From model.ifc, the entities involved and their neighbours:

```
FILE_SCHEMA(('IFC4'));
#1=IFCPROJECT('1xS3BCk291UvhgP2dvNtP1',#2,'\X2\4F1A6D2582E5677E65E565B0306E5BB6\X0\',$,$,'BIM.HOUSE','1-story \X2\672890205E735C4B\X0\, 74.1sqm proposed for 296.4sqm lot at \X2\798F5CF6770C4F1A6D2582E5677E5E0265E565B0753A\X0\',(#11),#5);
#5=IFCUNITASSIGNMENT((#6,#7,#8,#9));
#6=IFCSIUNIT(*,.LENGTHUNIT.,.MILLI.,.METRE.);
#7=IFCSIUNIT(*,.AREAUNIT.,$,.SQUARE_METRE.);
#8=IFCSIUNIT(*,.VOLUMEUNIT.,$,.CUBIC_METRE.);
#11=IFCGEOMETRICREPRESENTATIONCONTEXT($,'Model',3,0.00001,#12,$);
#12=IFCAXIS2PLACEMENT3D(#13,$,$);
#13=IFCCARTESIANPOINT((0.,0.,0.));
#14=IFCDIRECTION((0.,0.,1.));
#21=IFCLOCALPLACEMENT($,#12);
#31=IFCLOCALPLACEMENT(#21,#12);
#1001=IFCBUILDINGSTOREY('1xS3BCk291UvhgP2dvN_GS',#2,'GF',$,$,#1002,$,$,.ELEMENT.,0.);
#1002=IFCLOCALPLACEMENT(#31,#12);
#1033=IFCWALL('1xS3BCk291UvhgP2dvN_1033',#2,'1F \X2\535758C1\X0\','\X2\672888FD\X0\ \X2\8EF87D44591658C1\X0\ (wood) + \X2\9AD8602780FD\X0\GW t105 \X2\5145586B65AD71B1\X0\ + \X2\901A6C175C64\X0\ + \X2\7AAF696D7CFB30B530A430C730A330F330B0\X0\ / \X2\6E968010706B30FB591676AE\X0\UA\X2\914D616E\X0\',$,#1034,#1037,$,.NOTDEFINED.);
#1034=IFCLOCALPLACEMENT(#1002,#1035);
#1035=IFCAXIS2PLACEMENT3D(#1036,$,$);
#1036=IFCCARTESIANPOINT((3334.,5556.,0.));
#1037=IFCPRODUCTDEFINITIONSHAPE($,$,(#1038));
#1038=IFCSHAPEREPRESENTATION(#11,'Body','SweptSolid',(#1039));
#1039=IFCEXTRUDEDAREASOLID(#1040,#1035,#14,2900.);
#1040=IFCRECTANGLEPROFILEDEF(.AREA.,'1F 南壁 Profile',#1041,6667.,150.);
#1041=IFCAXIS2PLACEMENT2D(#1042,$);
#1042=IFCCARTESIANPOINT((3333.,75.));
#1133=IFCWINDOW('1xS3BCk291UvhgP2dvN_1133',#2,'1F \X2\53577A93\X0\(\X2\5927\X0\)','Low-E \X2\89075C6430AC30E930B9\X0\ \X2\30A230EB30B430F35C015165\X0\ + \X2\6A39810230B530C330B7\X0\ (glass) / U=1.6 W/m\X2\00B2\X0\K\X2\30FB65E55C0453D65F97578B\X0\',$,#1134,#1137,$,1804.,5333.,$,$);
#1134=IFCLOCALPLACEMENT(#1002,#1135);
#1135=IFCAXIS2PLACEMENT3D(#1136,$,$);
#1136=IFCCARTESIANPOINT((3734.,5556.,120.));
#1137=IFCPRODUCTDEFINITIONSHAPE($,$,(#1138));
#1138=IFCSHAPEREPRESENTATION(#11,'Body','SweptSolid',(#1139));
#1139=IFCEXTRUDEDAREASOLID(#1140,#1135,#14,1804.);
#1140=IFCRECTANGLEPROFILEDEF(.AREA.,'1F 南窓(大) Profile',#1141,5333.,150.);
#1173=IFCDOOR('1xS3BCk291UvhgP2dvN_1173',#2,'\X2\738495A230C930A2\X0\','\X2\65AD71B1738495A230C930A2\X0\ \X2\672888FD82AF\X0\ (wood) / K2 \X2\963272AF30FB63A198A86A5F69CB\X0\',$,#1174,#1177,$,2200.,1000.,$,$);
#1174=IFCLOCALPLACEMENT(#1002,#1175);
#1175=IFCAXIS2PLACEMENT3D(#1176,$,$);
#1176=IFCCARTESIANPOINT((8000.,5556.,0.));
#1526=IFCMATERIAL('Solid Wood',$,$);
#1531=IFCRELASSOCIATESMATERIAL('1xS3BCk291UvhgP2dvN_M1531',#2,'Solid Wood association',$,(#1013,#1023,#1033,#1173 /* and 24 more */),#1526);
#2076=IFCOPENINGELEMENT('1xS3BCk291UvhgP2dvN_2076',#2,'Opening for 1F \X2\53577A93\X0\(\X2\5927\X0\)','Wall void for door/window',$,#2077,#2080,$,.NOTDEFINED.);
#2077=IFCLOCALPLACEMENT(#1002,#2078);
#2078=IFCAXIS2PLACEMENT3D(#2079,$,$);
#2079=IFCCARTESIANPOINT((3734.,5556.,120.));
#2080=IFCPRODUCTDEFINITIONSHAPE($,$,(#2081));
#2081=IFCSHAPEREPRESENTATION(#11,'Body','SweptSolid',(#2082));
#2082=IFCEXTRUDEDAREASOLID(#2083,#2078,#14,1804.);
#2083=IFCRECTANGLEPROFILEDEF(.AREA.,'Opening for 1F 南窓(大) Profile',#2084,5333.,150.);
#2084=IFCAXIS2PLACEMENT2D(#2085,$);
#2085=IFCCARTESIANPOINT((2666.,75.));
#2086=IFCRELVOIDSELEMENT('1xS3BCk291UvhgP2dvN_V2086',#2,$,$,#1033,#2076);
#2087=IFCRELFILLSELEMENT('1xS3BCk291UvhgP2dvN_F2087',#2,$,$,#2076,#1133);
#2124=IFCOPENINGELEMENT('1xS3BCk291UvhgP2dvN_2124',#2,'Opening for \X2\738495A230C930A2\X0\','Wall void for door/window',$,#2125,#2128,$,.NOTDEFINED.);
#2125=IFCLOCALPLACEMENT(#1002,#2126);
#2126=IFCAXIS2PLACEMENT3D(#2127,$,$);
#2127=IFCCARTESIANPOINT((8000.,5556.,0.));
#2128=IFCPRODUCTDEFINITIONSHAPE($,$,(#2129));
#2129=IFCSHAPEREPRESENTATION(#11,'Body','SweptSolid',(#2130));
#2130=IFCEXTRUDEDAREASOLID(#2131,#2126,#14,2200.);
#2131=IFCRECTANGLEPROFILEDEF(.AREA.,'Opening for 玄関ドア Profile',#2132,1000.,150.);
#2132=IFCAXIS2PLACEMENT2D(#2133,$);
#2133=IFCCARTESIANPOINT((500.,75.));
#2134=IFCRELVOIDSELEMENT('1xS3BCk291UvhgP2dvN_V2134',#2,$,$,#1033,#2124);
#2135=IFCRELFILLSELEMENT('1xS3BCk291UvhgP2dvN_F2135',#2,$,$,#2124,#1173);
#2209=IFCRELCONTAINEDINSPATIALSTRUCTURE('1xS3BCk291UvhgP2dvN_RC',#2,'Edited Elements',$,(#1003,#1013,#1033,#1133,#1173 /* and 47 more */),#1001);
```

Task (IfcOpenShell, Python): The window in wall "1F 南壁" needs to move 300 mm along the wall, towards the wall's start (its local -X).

```python
import ifcopenshell
import ifcopenshell.api.geometry
import ifcopenshell.util.placement

model = ifcopenshell.open("model.ifc")

window = model.by_guid("1xS3BCk291UvhgP2dvN_1133")
opening = window.FillsVoids[0].RelatingOpeningElement
wall = opening.VoidsElements[0].RelatingBuildingElement

wall_matrix = ifcopenshell.util.placement.get_local_placement(wall.ObjectPlacement)
shift = wall_matrix[:3, 0] * -300.0
before = ifcopenshell.util.placement.get_local_placement(window.ObjectPlacement)[:3, 3].copy()

# The window is not placed relative to its opening, so move both.
for product in (opening, window):
    matrix = ifcopenshell.util.placement.get_local_placement(product.ObjectPlacement)
    matrix[:3, 3] += shift
    ifcopenshell.api.geometry.edit_object_placement(model, product=product, matrix=matrix, is_si=False)

after = ifcopenshell.util.placement.get_local_placement(window.ObjectPlacement)[:3, 3]
print("window moved by", (after - before).round(3) + 0.0)

model.write("model_rev.ifc")
```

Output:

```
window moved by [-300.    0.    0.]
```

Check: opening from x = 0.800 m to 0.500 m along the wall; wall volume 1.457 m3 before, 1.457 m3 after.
